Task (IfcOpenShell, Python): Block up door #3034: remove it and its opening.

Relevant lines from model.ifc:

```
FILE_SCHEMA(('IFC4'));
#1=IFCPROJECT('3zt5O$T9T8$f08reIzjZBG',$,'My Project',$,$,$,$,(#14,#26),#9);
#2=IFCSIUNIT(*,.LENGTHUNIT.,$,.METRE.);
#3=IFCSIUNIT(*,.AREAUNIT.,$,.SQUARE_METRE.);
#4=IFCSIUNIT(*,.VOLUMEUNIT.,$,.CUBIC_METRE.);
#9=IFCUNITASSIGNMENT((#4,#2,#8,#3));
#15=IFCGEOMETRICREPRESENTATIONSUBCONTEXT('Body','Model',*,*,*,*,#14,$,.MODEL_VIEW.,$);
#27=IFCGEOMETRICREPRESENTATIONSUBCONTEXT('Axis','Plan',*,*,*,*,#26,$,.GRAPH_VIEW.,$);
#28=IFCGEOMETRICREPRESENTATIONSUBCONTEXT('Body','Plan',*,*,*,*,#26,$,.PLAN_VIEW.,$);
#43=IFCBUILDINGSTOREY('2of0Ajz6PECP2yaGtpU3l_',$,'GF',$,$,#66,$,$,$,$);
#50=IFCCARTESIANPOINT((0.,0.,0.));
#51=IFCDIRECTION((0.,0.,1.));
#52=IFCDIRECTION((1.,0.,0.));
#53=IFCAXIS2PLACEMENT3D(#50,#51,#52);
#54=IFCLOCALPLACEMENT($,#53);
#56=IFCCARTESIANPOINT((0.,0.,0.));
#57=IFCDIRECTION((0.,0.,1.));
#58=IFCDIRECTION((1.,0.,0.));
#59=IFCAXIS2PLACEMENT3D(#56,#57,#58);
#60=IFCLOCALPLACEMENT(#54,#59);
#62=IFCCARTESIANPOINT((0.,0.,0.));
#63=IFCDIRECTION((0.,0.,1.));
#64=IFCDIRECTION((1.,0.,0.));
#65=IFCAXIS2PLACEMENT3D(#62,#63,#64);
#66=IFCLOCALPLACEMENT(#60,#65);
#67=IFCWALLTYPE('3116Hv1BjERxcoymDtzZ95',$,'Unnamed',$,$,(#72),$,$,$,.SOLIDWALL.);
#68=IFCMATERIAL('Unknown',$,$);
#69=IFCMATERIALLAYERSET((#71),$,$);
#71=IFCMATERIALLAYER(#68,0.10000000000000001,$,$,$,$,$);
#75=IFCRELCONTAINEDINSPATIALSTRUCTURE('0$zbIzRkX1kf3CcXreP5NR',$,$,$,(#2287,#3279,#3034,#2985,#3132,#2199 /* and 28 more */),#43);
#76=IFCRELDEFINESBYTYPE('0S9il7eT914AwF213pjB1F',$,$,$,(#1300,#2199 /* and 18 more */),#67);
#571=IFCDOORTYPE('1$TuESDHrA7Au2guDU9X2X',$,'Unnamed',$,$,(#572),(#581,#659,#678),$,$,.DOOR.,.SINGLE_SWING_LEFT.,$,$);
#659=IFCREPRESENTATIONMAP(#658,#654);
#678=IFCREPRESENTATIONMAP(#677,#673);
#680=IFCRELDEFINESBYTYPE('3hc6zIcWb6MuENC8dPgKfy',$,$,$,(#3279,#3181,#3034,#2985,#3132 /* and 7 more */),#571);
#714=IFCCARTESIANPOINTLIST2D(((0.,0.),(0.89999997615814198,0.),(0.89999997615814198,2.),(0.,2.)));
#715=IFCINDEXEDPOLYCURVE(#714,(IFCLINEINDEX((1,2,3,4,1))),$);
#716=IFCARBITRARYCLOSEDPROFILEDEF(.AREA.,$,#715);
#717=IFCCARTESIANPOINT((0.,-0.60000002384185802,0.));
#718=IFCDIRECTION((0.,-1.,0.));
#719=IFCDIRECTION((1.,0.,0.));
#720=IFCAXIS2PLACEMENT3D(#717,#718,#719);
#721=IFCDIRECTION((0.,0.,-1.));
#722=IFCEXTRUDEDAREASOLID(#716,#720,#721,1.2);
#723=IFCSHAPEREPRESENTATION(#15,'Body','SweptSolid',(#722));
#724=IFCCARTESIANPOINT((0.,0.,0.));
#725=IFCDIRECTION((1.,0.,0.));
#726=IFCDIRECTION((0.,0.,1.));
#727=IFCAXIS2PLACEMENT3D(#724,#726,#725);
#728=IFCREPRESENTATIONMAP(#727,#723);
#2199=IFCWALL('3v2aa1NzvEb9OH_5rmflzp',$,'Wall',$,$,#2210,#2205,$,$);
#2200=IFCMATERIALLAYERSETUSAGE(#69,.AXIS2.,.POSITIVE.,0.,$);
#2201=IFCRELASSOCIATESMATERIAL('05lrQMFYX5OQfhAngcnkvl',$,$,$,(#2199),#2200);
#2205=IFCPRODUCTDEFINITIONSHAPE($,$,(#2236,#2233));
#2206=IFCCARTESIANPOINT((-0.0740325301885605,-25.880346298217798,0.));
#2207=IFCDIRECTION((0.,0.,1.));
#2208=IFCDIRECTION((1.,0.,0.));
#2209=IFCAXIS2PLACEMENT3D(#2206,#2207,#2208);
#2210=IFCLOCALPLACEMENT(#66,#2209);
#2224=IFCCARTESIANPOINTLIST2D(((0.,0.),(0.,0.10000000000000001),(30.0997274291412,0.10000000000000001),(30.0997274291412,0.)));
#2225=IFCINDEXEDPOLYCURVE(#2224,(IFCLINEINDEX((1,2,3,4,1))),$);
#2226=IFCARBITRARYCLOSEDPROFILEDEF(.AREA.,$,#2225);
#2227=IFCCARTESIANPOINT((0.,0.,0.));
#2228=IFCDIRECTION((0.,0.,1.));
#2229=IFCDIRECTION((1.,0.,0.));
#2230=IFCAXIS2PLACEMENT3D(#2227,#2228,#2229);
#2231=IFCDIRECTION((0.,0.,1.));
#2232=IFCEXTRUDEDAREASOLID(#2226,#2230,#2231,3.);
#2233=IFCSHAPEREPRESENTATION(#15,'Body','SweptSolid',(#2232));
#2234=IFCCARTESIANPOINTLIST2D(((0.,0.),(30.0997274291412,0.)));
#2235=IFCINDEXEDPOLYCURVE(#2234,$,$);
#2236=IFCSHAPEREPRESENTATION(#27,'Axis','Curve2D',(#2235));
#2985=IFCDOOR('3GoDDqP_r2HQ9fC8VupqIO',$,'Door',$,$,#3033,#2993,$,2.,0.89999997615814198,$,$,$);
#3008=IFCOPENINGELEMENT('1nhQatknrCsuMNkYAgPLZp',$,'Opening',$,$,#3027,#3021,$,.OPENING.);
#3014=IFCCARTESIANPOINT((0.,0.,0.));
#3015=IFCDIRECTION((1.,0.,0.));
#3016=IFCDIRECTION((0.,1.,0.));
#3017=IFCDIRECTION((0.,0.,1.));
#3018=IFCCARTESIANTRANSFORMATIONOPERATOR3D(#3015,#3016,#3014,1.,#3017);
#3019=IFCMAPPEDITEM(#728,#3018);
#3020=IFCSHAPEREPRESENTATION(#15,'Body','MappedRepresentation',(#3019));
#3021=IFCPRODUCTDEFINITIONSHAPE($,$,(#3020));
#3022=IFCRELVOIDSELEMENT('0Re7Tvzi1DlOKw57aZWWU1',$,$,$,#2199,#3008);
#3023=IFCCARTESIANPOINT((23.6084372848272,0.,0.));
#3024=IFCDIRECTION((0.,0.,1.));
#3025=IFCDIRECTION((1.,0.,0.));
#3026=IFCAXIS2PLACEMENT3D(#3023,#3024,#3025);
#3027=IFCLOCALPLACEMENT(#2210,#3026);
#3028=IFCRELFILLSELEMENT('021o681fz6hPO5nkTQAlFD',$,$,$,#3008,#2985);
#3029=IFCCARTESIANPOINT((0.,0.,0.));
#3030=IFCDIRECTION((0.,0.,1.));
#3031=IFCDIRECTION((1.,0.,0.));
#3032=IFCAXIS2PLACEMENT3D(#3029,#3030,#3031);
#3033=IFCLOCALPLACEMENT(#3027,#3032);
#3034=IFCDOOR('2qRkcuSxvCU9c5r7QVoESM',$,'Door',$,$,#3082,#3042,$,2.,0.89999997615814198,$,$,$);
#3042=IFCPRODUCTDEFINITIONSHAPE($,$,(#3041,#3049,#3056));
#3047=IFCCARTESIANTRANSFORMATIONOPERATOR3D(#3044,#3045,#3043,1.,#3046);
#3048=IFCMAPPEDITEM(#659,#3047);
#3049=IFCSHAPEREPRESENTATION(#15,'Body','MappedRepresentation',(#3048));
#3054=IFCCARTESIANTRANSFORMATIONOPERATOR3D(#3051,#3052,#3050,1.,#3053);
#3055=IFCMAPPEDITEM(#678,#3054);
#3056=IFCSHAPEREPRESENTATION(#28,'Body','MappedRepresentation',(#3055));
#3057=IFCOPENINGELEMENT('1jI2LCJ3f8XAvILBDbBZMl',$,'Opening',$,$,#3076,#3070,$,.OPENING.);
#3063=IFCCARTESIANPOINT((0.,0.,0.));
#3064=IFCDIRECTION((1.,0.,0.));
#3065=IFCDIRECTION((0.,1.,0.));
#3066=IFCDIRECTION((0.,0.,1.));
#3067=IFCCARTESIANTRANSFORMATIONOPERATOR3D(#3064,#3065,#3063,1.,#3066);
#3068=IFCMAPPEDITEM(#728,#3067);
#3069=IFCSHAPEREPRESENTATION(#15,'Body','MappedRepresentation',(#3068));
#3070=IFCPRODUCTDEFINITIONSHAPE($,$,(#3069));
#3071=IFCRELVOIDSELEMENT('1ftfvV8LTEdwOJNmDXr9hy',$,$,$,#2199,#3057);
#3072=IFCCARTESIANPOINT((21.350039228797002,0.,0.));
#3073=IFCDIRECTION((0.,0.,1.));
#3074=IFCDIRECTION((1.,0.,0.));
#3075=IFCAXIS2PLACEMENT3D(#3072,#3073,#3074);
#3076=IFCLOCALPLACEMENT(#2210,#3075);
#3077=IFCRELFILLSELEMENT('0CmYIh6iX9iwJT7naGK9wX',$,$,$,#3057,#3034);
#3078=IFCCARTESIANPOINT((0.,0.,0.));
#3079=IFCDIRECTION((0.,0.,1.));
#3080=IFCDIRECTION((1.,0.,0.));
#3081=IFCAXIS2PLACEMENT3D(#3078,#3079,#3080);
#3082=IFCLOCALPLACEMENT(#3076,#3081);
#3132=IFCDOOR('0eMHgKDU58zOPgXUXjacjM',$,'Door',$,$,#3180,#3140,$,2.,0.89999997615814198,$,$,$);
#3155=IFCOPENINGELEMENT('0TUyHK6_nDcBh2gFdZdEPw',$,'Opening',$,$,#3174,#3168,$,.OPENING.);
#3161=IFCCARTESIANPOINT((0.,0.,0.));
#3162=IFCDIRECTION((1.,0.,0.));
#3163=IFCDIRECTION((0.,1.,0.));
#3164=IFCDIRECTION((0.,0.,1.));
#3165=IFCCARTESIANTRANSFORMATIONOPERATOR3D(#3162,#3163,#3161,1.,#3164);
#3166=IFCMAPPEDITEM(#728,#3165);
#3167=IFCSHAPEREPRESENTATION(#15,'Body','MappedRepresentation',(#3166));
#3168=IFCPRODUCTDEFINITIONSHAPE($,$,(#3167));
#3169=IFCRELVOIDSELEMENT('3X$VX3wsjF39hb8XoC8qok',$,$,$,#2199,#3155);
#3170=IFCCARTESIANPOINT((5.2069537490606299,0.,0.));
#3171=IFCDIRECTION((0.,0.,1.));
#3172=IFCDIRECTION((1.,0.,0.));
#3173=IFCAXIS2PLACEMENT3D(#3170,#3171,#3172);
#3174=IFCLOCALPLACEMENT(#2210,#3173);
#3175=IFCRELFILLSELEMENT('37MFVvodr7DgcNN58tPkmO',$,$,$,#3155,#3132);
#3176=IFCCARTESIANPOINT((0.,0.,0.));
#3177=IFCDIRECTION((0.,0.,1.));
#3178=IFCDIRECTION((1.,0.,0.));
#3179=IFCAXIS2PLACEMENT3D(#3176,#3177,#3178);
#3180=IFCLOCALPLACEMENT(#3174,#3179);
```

```python
import ifcopenshell
import ifcopenshell.api.feature
import ifcopenshell.api.root
import ifcopenshell.geom
import ifcopenshell.util.shape

model = ifcopenshell.open("model.ifc")
settings = ifcopenshell.geom.settings()


def volume(element):
    """Net volume in cubic metres, openings subtracted."""
    shape = ifcopenshell.geom.create_shape(settings, element)
    return ifcopenshell.util.shape.get_volume(shape.geometry)


door = model.by_id(3034)
opening = door.FillsVoids[0].RelatingOpeningElement
wall = opening.VoidsElements[0].RelatingBuildingElement
before = volume(wall)

ifcopenshell.api.root.remove_product(model, product=door)
ifcopenshell.api.feature.remove_feature(model, feature=opening)

after = volume(wall)

print(f"wall volume {before:.3f} -> {after:.3f} m3")

model.write("model_edited.ifc")
```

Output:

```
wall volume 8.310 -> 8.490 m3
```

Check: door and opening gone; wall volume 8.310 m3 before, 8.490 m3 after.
